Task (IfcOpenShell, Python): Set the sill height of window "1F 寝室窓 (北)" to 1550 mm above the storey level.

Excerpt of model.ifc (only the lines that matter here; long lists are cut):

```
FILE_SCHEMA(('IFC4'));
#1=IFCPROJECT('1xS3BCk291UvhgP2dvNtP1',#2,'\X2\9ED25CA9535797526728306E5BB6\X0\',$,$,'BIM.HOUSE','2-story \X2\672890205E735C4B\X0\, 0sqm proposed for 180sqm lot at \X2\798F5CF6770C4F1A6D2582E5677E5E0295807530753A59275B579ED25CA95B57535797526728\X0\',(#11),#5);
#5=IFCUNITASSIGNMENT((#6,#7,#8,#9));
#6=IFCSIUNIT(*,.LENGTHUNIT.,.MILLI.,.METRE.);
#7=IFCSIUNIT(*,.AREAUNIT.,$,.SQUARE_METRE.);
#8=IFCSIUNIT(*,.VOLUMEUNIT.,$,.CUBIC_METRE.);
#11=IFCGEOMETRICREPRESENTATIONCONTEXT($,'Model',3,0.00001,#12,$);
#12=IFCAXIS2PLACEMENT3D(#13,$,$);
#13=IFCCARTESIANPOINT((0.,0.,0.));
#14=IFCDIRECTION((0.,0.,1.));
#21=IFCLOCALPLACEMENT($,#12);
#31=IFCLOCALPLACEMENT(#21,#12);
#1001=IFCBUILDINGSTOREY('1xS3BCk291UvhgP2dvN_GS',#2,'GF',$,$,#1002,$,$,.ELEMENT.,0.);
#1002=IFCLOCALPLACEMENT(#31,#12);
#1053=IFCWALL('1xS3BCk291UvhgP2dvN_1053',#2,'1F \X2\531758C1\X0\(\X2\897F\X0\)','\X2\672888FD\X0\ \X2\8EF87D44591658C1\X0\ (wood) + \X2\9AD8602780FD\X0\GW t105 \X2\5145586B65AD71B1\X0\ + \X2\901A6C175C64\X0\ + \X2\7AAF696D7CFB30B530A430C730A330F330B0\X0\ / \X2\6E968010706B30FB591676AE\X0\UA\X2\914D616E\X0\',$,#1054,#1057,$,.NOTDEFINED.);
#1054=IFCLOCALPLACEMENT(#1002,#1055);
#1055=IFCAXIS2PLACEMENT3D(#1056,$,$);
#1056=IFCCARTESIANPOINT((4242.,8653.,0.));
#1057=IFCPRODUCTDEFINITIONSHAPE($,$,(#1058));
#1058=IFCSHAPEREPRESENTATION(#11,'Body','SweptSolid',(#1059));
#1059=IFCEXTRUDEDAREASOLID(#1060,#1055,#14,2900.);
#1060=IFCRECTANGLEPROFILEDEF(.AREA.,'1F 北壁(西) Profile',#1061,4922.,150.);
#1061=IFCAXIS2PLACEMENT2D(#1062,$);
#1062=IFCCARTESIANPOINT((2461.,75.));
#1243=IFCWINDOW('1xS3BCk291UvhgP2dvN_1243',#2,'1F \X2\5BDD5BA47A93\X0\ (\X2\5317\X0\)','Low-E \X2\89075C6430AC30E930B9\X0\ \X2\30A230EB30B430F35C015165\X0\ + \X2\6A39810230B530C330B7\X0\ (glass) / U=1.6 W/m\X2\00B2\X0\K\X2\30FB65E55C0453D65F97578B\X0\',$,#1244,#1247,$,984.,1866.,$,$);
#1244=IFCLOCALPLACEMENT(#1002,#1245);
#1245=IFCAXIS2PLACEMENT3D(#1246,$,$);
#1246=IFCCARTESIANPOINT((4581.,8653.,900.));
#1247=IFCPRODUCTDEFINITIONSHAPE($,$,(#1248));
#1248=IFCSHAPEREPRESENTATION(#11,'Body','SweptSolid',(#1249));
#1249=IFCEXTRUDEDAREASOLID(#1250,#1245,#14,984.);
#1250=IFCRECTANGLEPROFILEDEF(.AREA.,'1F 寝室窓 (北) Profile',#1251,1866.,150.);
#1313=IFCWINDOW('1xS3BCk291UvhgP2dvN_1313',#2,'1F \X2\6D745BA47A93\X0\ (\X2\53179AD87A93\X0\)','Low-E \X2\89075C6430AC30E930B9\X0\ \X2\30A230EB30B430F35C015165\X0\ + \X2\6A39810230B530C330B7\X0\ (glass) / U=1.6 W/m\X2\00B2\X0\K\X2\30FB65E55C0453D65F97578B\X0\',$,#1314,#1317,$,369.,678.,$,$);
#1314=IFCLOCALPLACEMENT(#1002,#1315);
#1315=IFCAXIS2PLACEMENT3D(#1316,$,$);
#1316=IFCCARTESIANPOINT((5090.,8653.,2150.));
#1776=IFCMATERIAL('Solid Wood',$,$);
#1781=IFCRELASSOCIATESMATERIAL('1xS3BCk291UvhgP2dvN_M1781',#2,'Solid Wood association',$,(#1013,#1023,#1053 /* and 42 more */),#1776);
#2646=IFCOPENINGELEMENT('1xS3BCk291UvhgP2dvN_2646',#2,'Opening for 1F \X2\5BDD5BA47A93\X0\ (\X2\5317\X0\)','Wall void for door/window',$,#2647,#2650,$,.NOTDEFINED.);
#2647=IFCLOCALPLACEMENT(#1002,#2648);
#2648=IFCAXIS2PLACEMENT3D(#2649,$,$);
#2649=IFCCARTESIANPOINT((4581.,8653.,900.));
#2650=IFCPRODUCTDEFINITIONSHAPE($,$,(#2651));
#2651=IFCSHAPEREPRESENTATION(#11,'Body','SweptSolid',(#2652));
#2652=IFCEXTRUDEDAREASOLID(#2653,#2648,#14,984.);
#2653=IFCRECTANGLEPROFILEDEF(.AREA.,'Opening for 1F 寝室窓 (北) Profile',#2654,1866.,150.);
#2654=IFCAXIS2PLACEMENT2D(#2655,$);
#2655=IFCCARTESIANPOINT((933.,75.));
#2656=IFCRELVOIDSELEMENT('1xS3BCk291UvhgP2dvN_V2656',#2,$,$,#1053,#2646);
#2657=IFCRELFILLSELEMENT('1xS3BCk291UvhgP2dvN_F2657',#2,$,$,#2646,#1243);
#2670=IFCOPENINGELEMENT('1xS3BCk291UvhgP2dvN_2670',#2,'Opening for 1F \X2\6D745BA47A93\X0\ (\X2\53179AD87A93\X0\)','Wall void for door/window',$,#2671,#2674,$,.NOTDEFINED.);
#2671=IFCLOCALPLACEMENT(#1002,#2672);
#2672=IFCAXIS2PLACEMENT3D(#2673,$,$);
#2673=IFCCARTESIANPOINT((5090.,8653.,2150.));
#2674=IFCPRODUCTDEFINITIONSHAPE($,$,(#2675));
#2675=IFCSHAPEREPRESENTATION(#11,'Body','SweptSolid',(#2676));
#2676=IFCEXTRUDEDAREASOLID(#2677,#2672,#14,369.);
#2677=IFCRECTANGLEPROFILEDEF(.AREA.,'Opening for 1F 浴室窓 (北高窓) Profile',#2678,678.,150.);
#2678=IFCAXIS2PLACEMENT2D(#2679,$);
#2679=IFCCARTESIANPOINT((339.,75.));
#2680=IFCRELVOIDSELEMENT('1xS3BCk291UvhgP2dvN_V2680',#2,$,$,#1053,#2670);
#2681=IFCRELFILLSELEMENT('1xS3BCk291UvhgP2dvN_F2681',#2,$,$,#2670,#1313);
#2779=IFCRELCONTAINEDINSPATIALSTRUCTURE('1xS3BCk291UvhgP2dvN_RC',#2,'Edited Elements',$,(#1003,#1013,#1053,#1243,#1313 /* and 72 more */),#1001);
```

```python
import numpy as np
import ifcopenshell
import ifcopenshell.api.geometry
import ifcopenshell.geom
import ifcopenshell.util.element
import ifcopenshell.util.placement
import ifcopenshell.util.shape
import ifcopenshell.util.unit

model = ifcopenshell.open("model.ifc")
unit_scale = ifcopenshell.util.unit.calculate_unit_scale(model)

window = model.by_id(1243)
opening = window.FillsVoids[0].RelatingOpeningElement
storey = ifcopenshell.util.element.get_container(window, ifc_class="IfcBuildingStorey")
level = ifcopenshell.util.placement.get_local_placement(storey.ObjectPlacement)[2, 3]

# The opening's origin need not be at the sill, so measure its lowest point.
shape = ifcopenshell.geom.create_shape(ifcopenshell.geom.settings(), opening)
bottom = ifcopenshell.util.shape.get_shape_bottom_elevation(shape, shape.geometry) / unit_scale
dz = level + 1550.0 - bottom

shift = np.array([0.0, 0.0, dz])
# The window is not placed relative to its opening, so move both.
for product in (opening, window):
    matrix = ifcopenshell.util.placement.get_local_placement(product.ObjectPlacement)
    matrix[:3, 3] += shift
    ifcopenshell.api.geometry.edit_object_placement(model, product=product, matrix=matrix, is_si=False)

print(f"moved by {dz * unit_scale:+.3f} m")

model.write("model_updated.ifc")
```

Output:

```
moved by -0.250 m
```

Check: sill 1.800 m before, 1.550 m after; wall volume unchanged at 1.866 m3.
